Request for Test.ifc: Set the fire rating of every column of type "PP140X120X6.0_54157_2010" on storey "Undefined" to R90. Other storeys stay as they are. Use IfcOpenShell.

First a look at what the model holds.

```python
import ifcopenshell
import ifcopenshell.util.element

model = ifcopenshell.open("Test.ifc")
print(model.schema)
storey = next(s for s in model.by_type("IfcBuildingStorey") if s.Name == "Undefined")
columns = [e for e in ifcopenshell.util.element.get_decomposition(storey) if e.is_a("IfcColumn")]
seen = {}
for e in columns:
    element_type = ifcopenshell.util.element.get_type(e)
    key = (element_type.Name if element_type != e and element_type else None, ifcopenshell.util.element.get_pset(e, "Pset_ColumnCommon", "FireRating"))
    seen[key] = seen.get(key, 0) + 1
for (name, value), count in sorted(seen.items(), key=str):
    print(count, "x", name, "|", value)
```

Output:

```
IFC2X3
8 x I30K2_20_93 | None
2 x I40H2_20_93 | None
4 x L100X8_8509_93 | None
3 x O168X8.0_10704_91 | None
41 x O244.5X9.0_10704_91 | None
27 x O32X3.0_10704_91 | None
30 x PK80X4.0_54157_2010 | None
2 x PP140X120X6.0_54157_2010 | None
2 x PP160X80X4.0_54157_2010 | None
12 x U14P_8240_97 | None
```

```python
import ifcopenshell
import ifcopenshell.api.pset
import ifcopenshell.util.element

model = ifcopenshell.open("Test.ifc")

storey = next(s for s in model.by_type("IfcBuildingStorey") if s.Name == "Undefined")
columns = [e for e in ifcopenshell.util.element.get_decomposition(storey) if e.is_a("IfcColumn")]

count = 0
for e in columns:
    element_type = ifcopenshell.util.element.get_type(e)
    if element_type in (None, e) or element_type.Name != "PP140X120X6.0_54157_2010":
        continue
    found = ifcopenshell.util.element.get_pset(e, "Pset_ColumnCommon", should_inherit=False)
    if found:
        pset = model.by_id(found["id"])
        if len(ifcopenshell.util.element.get_elements_by_pset(pset)) > 1:
            pset = ifcopenshell.api.pset.unshare_pset(model, products=[e], pset=pset)[0]
    else:
        pset = ifcopenshell.api.pset.add_pset(model, product=e, name="Pset_ColumnCommon")
    ifcopenshell.api.pset.edit_pset(model, pset=pset, properties={"FireRating": "R90"})
    count += 1

print(count, "columns updated")

model.write("Test_updated.ifc")
```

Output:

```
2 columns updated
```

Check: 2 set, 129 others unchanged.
